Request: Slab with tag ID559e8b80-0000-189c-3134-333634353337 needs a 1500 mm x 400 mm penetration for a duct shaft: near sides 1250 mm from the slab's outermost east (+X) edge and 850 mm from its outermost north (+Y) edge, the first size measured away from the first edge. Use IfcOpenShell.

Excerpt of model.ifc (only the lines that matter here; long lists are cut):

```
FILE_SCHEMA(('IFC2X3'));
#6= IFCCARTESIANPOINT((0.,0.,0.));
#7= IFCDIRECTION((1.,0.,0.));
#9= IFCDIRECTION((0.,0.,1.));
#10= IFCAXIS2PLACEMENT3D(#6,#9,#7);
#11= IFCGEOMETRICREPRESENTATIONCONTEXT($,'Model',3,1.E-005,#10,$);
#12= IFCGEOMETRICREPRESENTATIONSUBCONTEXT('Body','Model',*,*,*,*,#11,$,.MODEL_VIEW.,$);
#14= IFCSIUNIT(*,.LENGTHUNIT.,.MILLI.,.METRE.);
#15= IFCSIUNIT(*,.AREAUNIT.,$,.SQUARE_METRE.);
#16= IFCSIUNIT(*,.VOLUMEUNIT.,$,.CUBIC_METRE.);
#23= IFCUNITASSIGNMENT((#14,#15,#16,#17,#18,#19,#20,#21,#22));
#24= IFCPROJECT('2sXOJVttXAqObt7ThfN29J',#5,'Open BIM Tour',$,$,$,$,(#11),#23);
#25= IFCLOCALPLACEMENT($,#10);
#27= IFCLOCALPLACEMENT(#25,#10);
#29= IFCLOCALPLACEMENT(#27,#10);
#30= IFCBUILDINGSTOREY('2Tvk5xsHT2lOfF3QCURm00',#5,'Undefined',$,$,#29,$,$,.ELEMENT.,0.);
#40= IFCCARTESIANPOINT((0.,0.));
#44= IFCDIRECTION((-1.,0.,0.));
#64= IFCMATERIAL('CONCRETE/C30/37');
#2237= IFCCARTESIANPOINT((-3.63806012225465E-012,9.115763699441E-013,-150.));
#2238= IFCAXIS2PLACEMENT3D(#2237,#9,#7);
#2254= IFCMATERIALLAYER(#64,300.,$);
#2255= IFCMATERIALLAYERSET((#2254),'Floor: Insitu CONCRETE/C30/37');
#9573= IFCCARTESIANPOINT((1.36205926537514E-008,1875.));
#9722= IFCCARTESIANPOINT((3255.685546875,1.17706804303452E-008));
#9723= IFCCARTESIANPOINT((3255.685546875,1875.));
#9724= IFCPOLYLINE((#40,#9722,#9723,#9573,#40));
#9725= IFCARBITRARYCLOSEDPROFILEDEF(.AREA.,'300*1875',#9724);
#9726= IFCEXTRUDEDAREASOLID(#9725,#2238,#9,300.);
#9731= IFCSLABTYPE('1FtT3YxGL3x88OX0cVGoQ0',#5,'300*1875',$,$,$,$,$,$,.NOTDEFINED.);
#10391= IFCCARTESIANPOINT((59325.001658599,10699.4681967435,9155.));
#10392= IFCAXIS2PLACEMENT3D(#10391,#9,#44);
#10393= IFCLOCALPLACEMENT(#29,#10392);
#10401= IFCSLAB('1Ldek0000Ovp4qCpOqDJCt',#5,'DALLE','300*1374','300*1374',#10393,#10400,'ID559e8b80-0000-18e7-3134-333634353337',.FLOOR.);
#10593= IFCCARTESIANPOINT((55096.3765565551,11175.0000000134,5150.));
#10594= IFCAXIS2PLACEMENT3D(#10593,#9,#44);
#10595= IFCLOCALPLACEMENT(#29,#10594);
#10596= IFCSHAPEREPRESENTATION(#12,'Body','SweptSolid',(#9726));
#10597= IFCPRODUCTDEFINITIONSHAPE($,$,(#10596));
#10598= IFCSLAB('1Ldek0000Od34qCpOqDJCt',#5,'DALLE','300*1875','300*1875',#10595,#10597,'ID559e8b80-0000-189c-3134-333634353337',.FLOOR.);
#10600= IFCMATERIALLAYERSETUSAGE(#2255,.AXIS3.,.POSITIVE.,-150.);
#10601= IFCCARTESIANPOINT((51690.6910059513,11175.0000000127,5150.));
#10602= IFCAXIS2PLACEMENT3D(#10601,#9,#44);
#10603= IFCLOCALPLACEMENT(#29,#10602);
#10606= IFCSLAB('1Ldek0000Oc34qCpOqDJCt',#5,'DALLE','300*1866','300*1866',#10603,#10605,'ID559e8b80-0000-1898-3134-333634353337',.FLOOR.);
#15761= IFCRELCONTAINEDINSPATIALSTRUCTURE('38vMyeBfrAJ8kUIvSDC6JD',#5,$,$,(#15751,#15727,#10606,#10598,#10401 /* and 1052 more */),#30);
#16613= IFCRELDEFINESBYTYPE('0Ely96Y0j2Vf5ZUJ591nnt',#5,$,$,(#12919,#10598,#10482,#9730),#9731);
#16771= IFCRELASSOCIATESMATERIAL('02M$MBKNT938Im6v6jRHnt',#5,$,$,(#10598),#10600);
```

```python
import numpy as np
import ifcopenshell
import ifcopenshell.api.feature
import ifcopenshell.api.geometry
import ifcopenshell.api.root
import ifcopenshell.geom
import ifcopenshell.util.placement
import ifcopenshell.util.representation
import ifcopenshell.util.shape
import ifcopenshell.util.unit

model = ifcopenshell.open("model.ifc")
unit_scale = ifcopenshell.util.unit.calculate_unit_scale(model)
settings = ifcopenshell.geom.settings()


def volume(element):
    """Net volume in cubic metres, openings subtracted."""
    shape = ifcopenshell.geom.create_shape(settings, element)
    return ifcopenshell.util.shape.get_volume(shape.geometry)


slab = model.by_guid("1Ldek0000Od34qCpOqDJCt")
before = volume(slab)

# Extent in the slab's own axes, in metres. The edges named are its -X and -Y sides.
slab_shape = ifcopenshell.geom.create_shape(settings, slab)
vertices = ifcopenshell.util.shape.get_vertices(slab_shape.geometry)
x_min, y_min, bottom = vertices.min(axis=0)
top = vertices[:, 2].max()

opening = ifcopenshell.api.root.create_entity(model, ifc_class="IfcOpeningElement", name="Duct shaft opening")
context = ifcopenshell.util.representation.get_context(model, "Model", "Body", "MODEL_VIEW")
width, depth = 1.5, 0.4
outline = [(0.0, 0.0), (width, 0.0), (width, depth), (0.0, depth), (0.0, 0.0)]
# Overshoot both faces by 50 mm so the cut is clean.
shape = ifcopenshell.api.geometry.add_slab_representation(
    model, context=context, depth=top - bottom + 0.1, polyline=outline
)
ifcopenshell.api.geometry.assign_representation(model, product=opening, representation=shape)

matrix = ifcopenshell.util.placement.get_local_placement(slab.ObjectPlacement)
matrix[:, 3] = matrix @ np.append(np.array([x_min + 1.25, y_min + 0.85, bottom - 0.05]) / unit_scale, 1.0)
ifcopenshell.api.geometry.edit_object_placement(model, product=opening, matrix=matrix, is_si=False)
ifcopenshell.api.feature.add_feature(model, feature=opening, element=slab)

after = volume(slab)

print(f"slab volume {before:.3f} -> {after:.3f} m3")

model.write("model_edited.ifc")
```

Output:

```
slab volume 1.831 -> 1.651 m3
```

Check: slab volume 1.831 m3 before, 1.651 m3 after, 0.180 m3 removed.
